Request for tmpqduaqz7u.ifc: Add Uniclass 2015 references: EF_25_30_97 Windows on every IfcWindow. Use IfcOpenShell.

First a look at what the model holds.

```python
import ifcopenshell

model = ifcopenshell.open("tmpqduaqz7u.ifc")
print(model.schema)
print("classifications:", [c.Name for c in model.by_type("IfcClassification")])
for ifc_class in ("IfcDoor", "IfcRoof", "IfcStair", "IfcWall", "IfcWindow"):
    print(ifc_class, len(model.by_type(ifc_class)))
```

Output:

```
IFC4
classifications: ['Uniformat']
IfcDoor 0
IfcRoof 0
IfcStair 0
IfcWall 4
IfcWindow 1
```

```python
import ifcopenshell
import ifcopenshell.api.classification

model = ifcopenshell.open("tmpqduaqz7u.ifc")

system = ifcopenshell.api.classification.add_classification(model, classification="Uniclass 2015")

codes = {
    "IfcWindow": ("EF_25_30_97", "Windows"),
}
for ifc_class, (code, name) in codes.items():
    products = model.by_type(ifc_class)
    ifcopenshell.api.classification.add_reference(
        model, products=products, classification=system, identification=code, name=name
    )
    print(code, len(products))

model.write("tmpqduaqz7u_v2.ifc")
```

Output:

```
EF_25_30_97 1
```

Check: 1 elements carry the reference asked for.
